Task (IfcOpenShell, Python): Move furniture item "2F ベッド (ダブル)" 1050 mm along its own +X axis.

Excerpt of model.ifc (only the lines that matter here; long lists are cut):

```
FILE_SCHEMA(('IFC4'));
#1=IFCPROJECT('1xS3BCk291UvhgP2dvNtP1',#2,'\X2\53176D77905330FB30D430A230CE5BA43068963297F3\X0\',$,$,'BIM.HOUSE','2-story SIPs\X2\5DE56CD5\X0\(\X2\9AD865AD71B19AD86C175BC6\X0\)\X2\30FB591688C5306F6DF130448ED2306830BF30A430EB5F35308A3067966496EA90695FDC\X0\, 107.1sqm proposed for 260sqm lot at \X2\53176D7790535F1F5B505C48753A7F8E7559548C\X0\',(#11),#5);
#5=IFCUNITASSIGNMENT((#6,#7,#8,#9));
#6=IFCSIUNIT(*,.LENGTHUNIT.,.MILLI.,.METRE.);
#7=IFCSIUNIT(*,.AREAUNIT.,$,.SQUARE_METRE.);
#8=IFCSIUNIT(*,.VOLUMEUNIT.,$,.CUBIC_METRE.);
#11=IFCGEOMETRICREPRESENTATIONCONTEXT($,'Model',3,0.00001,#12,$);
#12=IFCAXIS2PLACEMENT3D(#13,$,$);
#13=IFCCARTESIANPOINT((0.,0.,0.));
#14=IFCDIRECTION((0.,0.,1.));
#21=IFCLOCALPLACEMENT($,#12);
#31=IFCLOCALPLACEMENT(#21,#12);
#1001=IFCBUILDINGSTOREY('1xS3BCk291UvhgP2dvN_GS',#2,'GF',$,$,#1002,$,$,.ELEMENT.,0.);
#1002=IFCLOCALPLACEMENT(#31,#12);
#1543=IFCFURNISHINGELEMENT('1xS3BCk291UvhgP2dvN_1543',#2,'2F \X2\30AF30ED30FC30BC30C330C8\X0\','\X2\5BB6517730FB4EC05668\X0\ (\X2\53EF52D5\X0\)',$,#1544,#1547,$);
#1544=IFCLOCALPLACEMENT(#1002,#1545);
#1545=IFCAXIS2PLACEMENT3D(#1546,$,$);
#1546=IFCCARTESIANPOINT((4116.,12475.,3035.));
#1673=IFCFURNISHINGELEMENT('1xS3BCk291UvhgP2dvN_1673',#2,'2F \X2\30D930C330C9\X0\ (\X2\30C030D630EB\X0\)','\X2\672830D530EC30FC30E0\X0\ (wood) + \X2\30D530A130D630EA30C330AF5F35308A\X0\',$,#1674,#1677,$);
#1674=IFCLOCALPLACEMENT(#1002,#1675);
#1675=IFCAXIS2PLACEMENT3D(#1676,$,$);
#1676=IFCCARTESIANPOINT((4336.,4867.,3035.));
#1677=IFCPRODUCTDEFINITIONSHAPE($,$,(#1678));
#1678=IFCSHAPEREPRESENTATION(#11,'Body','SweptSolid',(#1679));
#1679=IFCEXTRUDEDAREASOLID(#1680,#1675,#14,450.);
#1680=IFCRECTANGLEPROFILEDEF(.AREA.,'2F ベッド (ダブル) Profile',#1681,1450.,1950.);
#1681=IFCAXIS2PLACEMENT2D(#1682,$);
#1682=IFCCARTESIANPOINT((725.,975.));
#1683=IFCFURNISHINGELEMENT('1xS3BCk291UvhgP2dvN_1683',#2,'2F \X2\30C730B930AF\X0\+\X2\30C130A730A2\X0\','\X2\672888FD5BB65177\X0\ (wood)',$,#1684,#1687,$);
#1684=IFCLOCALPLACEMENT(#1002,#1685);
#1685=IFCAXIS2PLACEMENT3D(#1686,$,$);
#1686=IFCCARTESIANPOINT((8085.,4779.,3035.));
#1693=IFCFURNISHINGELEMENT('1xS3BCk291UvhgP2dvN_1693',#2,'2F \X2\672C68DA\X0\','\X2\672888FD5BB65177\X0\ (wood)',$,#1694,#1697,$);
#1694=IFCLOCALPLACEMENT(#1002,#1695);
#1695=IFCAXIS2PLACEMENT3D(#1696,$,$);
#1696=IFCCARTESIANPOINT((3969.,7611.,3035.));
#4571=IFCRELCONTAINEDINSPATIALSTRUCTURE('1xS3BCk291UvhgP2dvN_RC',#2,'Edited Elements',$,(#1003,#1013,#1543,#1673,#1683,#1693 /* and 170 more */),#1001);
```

```python
import ifcopenshell
import ifcopenshell.api.geometry
import ifcopenshell.util.placement

model = ifcopenshell.open("model.ifc")

item = model.by_guid("1xS3BCk291UvhgP2dvN_1673")
matrix = ifcopenshell.util.placement.get_local_placement(item.ObjectPlacement)
matrix[:3, 3] += matrix[:3, 0] * 1050.0
ifcopenshell.api.geometry.edit_object_placement(model, product=item, matrix=matrix, is_si=False)

print(ifcopenshell.util.placement.get_local_placement(item.ObjectPlacement).round(3) + 0.0)

model.write("model_updated.ifc")
```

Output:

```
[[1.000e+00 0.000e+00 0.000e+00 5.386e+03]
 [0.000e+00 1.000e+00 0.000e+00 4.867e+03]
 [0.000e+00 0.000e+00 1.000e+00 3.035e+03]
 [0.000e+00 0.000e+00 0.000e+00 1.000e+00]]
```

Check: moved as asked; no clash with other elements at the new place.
